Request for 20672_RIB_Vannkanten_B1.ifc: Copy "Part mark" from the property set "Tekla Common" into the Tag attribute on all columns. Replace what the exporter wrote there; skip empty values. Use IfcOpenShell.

First a look at what the model holds.

```python
import ifcopenshell
import ifcopenshell.util.element

model = ifcopenshell.open("20672_RIB_Vannkanten_B1.ifc")
print(model.schema)
columns = model.by_type("IfcColumn")
print(len(columns), "columns")
for e in columns[:8]:
    source = ifcopenshell.util.element.get_pset(e, "Tekla Common", "Part mark")
    target = e.Tag
    print(e.id(), repr(source), repr(target), sep=" | ")
```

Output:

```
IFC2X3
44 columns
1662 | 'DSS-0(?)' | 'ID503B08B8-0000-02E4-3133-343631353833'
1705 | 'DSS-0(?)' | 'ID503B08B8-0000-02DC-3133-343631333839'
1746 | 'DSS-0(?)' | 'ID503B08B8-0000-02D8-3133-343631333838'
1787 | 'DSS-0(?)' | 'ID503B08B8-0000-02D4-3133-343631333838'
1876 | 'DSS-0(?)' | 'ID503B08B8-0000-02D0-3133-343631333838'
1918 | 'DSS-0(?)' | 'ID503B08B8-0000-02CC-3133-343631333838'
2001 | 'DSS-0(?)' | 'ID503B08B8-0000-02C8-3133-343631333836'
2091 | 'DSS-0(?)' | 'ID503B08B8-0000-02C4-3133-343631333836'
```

```python
import ifcopenshell
import ifcopenshell.util.element

model = ifcopenshell.open("20672_RIB_Vannkanten_B1.ifc")

count = 0
for e in model.by_type("IfcColumn"):
    value = ifcopenshell.util.element.get_pset(e, "Tekla Common", "Part mark")
    current = e.Tag
    if not value or not value.strip() or current == value:
        continue
    e.Tag = value
    count += 1

print(count, "columns updated")

model.write("20672_RIB_Vannkanten_B1_v2.ifc")
```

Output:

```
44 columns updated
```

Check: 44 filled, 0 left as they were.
